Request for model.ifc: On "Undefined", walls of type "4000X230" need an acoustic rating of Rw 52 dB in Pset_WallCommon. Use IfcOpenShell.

First a look at what the model holds.

```python
import ifcopenshell
import ifcopenshell.util.element

model = ifcopenshell.open("model.ifc")
print(model.schema)
storey = next(s for s in model.by_type("IfcBuildingStorey") if s.Name == "Undefined")
walls = [e for e in ifcopenshell.util.element.get_decomposition(storey) if e.is_a("IfcWall")]
seen = {}
for e in walls:
    element_type = ifcopenshell.util.element.get_type(e)
    key = (element_type.Name if element_type != e and element_type else None, ifcopenshell.util.element.get_pset(e, "Pset_WallCommon", "AcousticRating"))
    seen[key] = seen.get(key, 0) + 1
for (name, value), count in sorted(seen.items(), key=str):
    print(count, "x", name, "|", value)
```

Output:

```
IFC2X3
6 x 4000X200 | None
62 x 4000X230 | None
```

```python
import ifcopenshell
import ifcopenshell.api.pset
import ifcopenshell.util.element

model = ifcopenshell.open("model.ifc")

storey = next(s for s in model.by_type("IfcBuildingStorey") if s.Name == "Undefined")
walls = [e for e in ifcopenshell.util.element.get_decomposition(storey) if e.is_a("IfcWall")]

count = 0
for e in walls:
    element_type = ifcopenshell.util.element.get_type(e)
    if element_type in (None, e) or element_type.Name != "4000X230":
        continue
    # add_pset returns the element's existing set when there is one.
    pset = ifcopenshell.api.pset.add_pset(model, product=e, name="Pset_WallCommon")
    ifcopenshell.api.pset.edit_pset(model, pset=pset, properties={"AcousticRating": "Rw 52 dB"})
    count += 1

print(count, "walls updated")

model.write("model_updated.ifc")
```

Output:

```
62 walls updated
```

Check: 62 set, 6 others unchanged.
